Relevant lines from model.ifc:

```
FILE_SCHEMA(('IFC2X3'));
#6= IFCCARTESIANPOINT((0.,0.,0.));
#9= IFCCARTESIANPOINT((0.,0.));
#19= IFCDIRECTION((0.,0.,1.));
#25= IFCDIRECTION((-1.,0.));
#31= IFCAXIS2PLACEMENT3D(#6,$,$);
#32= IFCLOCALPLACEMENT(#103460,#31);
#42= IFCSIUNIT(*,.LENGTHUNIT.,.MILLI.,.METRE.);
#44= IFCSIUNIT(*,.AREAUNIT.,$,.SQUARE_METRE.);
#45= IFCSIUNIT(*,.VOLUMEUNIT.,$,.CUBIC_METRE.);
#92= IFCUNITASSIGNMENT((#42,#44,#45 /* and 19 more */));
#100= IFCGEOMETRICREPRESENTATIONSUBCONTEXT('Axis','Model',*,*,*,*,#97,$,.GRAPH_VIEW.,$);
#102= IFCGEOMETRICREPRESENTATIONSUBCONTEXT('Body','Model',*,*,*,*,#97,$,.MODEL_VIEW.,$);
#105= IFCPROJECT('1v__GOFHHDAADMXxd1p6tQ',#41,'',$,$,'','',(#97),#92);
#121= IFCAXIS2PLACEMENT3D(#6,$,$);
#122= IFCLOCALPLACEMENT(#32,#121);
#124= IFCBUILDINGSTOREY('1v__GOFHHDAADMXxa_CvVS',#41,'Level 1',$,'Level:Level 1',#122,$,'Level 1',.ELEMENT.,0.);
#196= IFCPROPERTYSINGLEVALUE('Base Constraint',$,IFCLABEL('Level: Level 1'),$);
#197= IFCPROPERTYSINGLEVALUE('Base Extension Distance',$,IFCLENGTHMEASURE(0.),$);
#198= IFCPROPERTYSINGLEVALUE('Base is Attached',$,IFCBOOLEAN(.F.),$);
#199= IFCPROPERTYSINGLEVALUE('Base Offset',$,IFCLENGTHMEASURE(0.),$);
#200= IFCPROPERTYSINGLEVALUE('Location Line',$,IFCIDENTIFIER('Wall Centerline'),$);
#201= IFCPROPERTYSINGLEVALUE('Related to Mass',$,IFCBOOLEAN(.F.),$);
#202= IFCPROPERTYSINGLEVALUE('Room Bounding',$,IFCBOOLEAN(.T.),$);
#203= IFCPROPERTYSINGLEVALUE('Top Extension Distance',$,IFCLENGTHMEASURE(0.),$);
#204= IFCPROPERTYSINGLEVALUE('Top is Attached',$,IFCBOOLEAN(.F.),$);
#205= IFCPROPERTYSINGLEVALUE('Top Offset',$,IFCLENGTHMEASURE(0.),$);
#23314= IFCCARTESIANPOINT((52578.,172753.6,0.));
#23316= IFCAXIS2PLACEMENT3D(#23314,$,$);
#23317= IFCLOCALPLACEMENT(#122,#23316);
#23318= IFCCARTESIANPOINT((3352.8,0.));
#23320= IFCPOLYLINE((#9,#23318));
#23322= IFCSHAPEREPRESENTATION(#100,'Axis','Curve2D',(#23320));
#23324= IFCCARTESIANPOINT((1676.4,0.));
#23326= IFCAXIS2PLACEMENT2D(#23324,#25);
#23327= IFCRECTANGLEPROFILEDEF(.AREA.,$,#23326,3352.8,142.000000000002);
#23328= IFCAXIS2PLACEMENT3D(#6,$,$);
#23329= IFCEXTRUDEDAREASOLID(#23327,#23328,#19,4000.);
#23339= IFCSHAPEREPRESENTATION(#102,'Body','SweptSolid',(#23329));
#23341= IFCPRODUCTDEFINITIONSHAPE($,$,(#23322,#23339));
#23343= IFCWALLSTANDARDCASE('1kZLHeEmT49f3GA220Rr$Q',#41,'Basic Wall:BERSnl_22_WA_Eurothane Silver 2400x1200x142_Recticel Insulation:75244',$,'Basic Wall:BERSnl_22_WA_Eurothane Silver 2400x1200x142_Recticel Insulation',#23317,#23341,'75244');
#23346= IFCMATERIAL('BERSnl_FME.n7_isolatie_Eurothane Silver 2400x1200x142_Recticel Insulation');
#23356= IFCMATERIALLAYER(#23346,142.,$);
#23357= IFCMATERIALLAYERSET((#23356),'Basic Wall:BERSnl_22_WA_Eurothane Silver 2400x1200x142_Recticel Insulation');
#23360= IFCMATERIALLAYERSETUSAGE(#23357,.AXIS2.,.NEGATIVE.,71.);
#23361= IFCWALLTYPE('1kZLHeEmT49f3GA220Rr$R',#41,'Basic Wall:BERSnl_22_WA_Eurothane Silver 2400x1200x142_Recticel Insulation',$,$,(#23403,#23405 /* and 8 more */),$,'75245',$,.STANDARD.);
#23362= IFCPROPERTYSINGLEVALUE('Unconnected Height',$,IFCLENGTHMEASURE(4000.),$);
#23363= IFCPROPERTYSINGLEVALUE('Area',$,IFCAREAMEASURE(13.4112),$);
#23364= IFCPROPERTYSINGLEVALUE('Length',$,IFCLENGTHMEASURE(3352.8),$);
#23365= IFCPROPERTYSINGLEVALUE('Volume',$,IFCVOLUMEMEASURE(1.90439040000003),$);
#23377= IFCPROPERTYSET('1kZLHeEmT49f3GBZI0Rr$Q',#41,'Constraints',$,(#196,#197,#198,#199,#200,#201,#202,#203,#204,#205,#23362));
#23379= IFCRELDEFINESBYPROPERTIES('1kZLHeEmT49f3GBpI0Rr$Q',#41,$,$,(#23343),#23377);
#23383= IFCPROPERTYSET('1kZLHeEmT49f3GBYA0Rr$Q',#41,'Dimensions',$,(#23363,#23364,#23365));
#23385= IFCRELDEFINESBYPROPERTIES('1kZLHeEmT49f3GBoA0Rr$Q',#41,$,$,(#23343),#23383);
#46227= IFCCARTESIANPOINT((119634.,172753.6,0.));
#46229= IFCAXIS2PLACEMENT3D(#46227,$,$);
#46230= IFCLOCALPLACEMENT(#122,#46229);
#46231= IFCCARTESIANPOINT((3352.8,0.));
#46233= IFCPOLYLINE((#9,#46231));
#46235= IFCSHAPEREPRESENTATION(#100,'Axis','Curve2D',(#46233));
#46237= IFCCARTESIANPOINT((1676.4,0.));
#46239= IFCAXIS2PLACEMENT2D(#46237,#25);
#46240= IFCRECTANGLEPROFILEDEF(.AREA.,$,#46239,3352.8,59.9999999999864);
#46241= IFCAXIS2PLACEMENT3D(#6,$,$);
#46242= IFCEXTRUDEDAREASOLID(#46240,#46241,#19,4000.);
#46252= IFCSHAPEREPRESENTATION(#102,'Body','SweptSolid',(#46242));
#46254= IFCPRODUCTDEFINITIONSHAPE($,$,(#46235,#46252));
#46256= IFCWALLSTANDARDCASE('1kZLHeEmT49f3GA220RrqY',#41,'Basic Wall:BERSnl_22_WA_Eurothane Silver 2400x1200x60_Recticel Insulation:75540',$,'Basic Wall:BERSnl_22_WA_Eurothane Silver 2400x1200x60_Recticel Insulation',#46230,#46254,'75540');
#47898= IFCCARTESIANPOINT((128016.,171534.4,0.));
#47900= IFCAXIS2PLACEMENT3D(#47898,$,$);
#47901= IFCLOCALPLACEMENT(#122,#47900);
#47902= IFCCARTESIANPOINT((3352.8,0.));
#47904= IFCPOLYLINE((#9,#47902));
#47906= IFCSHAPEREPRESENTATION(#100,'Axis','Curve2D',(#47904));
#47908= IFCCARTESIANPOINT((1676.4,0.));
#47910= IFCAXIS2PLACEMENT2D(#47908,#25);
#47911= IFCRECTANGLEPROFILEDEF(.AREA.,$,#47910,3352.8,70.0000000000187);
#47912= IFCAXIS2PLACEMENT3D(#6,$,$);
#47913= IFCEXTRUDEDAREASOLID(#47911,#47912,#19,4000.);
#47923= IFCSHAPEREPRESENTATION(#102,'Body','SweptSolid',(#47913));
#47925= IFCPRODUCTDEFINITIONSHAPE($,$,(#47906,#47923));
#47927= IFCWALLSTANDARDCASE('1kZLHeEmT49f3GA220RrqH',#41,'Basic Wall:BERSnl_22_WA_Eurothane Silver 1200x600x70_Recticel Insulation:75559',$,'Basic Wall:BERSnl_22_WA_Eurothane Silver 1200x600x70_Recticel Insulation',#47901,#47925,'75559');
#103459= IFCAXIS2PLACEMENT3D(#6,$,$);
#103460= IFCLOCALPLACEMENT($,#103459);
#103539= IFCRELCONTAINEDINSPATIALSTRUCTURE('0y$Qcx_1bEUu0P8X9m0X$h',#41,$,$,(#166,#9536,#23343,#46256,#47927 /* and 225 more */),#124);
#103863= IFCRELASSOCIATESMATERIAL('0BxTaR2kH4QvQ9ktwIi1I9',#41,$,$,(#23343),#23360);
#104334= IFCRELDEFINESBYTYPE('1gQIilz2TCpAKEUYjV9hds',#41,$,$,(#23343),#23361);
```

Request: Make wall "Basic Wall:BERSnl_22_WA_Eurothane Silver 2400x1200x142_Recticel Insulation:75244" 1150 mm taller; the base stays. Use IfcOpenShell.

```python
import ifcopenshell
import ifcopenshell.api.pset
import ifcopenshell.geom
import ifcopenshell.util.element
import ifcopenshell.util.representation
import ifcopenshell.util.shape
import ifcopenshell.util.unit

model = ifcopenshell.open("model.ifc")
unit_scale = ifcopenshell.util.unit.calculate_unit_scale(model)
area_scale = ifcopenshell.util.unit.calculate_unit_scale(model, "AREAUNIT")
volume_scale = ifcopenshell.util.unit.calculate_unit_scale(model, "VOLUMEUNIT")
settings = ifcopenshell.geom.settings()


def volume(element):
    """Net volume in cubic metres, openings subtracted."""
    shape = ifcopenshell.geom.create_shape(settings, element)
    return ifcopenshell.util.shape.get_volume(shape.geometry)


wall = model.by_id(23343)
before = volume(wall)

body = ifcopenshell.util.representation.get_representation(wall, "Model", "Body")
solid = body.Items[0]
old_height = solid.Depth
solid.Depth += 1.15 / unit_scale
after = volume(wall)
thickness = 0.142  # wall thickness in metres

# Update the stored height, areas and volumes.
pset = model.by_id(ifcopenshell.util.element.get_pset(wall, "Constraints", should_inherit=False)["id"])
ifcopenshell.api.pset.edit_pset(model, pset=pset, properties={
    "Unconnected Height": model.create_entity("IfcLengthMeasure", solid.Depth),
})
pset = model.by_id(ifcopenshell.util.element.get_pset(wall, "Dimensions", should_inherit=False)["id"])
ifcopenshell.api.pset.edit_pset(model, pset=pset, properties={
    "Area": model.create_entity("IfcAreaMeasure", after / thickness / area_scale),
    "Volume": model.create_entity("IfcVolumeMeasure", after / volume_scale),
})

print(f"height {old_height:g} -> {solid.Depth:g}, volume {before:.3f} -> {after:.3f} m3")

model.write("model_rev.ifc")
```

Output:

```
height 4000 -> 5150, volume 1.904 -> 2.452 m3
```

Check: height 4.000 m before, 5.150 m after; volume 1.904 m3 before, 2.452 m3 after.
